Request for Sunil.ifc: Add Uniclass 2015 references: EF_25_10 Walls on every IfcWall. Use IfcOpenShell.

First a look at what the model holds.

```python
import ifcopenshell

model = ifcopenshell.open("Sunil.ifc")
print(model.schema)
print("classifications:", [c.Name for c in model.by_type("IfcClassification")])
for ifc_class in ("IfcDoor", "IfcRoof", "IfcStair", "IfcWall", "IfcWindow"):
    print(ifc_class, len(model.by_type(ifc_class)))
```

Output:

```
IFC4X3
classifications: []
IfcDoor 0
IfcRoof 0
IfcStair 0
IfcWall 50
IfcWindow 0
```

```python
import ifcopenshell
import ifcopenshell.api.classification

model = ifcopenshell.open("Sunil.ifc")

system = ifcopenshell.api.classification.add_classification(model, classification="Uniclass 2015")

codes = {
    "IfcWall": ("EF_25_10", "Walls"),
}
for ifc_class, (code, name) in codes.items():
    products = model.by_type(ifc_class)
    ifcopenshell.api.classification.add_reference(
        model, products=products, classification=system, identification=code, name=name
    )
    print(code, len(products))

model.write("Sunil_updated.ifc")
```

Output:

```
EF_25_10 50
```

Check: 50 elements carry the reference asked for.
